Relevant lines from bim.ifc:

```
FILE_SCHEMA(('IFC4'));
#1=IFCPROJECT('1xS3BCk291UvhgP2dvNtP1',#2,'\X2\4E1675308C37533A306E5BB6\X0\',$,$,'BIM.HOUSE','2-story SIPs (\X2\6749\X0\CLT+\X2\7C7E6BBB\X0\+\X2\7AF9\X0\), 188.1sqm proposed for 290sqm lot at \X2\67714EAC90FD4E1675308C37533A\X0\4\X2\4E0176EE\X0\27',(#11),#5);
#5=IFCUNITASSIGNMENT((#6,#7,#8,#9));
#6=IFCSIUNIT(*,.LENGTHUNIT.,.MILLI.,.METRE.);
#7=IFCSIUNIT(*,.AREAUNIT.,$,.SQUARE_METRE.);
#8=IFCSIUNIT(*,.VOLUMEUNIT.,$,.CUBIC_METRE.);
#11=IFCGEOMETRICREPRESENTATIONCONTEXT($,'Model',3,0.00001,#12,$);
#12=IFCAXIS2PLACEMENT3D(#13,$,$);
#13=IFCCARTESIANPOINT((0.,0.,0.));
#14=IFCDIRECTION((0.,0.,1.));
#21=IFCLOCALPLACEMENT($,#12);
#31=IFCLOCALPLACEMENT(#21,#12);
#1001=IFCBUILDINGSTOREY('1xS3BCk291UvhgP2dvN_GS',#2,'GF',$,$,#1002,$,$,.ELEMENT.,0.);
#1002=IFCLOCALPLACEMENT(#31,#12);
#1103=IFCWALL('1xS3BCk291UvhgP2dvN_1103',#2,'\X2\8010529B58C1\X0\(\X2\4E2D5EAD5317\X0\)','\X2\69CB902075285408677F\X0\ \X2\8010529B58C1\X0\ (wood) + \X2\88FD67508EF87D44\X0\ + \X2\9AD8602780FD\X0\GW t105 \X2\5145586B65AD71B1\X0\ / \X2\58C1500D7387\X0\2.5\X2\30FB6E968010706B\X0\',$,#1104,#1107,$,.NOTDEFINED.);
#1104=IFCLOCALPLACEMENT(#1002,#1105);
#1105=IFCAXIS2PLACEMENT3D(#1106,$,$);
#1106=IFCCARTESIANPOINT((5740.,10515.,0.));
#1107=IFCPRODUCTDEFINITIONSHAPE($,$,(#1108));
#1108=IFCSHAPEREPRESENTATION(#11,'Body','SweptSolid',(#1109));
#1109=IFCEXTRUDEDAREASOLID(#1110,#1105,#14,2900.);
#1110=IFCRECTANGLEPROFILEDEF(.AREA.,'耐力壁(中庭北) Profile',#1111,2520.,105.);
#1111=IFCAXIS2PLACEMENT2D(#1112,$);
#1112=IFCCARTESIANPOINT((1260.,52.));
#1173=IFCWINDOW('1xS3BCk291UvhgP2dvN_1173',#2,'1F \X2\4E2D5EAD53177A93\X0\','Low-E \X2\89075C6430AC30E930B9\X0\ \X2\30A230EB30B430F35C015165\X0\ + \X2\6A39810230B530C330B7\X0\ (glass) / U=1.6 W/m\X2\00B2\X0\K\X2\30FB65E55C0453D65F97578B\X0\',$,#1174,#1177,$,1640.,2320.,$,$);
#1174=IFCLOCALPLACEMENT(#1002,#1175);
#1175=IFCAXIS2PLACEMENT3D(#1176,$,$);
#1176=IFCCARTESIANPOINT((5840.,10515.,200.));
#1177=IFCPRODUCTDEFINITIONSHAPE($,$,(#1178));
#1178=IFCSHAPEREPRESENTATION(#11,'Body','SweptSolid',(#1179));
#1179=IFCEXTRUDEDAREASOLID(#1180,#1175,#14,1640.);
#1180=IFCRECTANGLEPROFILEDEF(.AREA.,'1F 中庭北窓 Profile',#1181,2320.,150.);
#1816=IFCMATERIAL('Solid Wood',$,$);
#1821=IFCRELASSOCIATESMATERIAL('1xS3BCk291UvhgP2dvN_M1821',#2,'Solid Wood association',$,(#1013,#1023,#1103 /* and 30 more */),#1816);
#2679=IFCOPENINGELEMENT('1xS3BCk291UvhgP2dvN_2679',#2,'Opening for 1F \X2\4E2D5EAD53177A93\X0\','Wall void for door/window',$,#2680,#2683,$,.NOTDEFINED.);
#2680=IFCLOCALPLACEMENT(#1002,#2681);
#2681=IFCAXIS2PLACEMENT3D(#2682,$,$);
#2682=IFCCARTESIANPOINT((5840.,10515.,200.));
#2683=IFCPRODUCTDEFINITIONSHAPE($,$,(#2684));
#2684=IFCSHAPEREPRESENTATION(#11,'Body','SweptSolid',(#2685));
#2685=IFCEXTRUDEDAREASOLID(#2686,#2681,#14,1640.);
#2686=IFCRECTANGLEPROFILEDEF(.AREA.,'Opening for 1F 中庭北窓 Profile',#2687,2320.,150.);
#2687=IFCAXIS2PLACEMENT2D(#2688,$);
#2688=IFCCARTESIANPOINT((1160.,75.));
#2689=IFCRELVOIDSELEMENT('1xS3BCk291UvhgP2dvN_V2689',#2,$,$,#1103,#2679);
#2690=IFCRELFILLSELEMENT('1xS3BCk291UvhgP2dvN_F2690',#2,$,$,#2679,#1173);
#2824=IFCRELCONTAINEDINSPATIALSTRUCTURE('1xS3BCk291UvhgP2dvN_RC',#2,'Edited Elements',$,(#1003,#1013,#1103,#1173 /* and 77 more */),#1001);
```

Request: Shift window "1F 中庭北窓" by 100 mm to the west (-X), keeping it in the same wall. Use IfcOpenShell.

```python
import ifcopenshell
import ifcopenshell.api.geometry
import ifcopenshell.util.placement
import ifcopenshell.util.unit

model = ifcopenshell.open("bim.ifc")
unit_scale = ifcopenshell.util.unit.calculate_unit_scale(model)

window = model.by_guid("1xS3BCk291UvhgP2dvN_1173")
opening = window.FillsVoids[0].RelatingOpeningElement
wall = opening.VoidsElements[0].RelatingBuildingElement

wall_matrix = ifcopenshell.util.placement.get_local_placement(wall.ObjectPlacement)
shift = wall_matrix[:3, 0] * -0.1 / unit_scale
before = ifcopenshell.util.placement.get_local_placement(window.ObjectPlacement)[:3, 3].copy()

# The window is not placed relative to its opening, so move both.
for product in (opening, window):
    matrix = ifcopenshell.util.placement.get_local_placement(product.ObjectPlacement)
    matrix[:3, 3] += shift
    ifcopenshell.api.geometry.edit_object_placement(model, product=product, matrix=matrix, is_si=False)

after = ifcopenshell.util.placement.get_local_placement(window.ObjectPlacement)[:3, 3]
print("window moved by", (after - before).round(3) + 0.0)

model.write("bim_rev.ifc")
```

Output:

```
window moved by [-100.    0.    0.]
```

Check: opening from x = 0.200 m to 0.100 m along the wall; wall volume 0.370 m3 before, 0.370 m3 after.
